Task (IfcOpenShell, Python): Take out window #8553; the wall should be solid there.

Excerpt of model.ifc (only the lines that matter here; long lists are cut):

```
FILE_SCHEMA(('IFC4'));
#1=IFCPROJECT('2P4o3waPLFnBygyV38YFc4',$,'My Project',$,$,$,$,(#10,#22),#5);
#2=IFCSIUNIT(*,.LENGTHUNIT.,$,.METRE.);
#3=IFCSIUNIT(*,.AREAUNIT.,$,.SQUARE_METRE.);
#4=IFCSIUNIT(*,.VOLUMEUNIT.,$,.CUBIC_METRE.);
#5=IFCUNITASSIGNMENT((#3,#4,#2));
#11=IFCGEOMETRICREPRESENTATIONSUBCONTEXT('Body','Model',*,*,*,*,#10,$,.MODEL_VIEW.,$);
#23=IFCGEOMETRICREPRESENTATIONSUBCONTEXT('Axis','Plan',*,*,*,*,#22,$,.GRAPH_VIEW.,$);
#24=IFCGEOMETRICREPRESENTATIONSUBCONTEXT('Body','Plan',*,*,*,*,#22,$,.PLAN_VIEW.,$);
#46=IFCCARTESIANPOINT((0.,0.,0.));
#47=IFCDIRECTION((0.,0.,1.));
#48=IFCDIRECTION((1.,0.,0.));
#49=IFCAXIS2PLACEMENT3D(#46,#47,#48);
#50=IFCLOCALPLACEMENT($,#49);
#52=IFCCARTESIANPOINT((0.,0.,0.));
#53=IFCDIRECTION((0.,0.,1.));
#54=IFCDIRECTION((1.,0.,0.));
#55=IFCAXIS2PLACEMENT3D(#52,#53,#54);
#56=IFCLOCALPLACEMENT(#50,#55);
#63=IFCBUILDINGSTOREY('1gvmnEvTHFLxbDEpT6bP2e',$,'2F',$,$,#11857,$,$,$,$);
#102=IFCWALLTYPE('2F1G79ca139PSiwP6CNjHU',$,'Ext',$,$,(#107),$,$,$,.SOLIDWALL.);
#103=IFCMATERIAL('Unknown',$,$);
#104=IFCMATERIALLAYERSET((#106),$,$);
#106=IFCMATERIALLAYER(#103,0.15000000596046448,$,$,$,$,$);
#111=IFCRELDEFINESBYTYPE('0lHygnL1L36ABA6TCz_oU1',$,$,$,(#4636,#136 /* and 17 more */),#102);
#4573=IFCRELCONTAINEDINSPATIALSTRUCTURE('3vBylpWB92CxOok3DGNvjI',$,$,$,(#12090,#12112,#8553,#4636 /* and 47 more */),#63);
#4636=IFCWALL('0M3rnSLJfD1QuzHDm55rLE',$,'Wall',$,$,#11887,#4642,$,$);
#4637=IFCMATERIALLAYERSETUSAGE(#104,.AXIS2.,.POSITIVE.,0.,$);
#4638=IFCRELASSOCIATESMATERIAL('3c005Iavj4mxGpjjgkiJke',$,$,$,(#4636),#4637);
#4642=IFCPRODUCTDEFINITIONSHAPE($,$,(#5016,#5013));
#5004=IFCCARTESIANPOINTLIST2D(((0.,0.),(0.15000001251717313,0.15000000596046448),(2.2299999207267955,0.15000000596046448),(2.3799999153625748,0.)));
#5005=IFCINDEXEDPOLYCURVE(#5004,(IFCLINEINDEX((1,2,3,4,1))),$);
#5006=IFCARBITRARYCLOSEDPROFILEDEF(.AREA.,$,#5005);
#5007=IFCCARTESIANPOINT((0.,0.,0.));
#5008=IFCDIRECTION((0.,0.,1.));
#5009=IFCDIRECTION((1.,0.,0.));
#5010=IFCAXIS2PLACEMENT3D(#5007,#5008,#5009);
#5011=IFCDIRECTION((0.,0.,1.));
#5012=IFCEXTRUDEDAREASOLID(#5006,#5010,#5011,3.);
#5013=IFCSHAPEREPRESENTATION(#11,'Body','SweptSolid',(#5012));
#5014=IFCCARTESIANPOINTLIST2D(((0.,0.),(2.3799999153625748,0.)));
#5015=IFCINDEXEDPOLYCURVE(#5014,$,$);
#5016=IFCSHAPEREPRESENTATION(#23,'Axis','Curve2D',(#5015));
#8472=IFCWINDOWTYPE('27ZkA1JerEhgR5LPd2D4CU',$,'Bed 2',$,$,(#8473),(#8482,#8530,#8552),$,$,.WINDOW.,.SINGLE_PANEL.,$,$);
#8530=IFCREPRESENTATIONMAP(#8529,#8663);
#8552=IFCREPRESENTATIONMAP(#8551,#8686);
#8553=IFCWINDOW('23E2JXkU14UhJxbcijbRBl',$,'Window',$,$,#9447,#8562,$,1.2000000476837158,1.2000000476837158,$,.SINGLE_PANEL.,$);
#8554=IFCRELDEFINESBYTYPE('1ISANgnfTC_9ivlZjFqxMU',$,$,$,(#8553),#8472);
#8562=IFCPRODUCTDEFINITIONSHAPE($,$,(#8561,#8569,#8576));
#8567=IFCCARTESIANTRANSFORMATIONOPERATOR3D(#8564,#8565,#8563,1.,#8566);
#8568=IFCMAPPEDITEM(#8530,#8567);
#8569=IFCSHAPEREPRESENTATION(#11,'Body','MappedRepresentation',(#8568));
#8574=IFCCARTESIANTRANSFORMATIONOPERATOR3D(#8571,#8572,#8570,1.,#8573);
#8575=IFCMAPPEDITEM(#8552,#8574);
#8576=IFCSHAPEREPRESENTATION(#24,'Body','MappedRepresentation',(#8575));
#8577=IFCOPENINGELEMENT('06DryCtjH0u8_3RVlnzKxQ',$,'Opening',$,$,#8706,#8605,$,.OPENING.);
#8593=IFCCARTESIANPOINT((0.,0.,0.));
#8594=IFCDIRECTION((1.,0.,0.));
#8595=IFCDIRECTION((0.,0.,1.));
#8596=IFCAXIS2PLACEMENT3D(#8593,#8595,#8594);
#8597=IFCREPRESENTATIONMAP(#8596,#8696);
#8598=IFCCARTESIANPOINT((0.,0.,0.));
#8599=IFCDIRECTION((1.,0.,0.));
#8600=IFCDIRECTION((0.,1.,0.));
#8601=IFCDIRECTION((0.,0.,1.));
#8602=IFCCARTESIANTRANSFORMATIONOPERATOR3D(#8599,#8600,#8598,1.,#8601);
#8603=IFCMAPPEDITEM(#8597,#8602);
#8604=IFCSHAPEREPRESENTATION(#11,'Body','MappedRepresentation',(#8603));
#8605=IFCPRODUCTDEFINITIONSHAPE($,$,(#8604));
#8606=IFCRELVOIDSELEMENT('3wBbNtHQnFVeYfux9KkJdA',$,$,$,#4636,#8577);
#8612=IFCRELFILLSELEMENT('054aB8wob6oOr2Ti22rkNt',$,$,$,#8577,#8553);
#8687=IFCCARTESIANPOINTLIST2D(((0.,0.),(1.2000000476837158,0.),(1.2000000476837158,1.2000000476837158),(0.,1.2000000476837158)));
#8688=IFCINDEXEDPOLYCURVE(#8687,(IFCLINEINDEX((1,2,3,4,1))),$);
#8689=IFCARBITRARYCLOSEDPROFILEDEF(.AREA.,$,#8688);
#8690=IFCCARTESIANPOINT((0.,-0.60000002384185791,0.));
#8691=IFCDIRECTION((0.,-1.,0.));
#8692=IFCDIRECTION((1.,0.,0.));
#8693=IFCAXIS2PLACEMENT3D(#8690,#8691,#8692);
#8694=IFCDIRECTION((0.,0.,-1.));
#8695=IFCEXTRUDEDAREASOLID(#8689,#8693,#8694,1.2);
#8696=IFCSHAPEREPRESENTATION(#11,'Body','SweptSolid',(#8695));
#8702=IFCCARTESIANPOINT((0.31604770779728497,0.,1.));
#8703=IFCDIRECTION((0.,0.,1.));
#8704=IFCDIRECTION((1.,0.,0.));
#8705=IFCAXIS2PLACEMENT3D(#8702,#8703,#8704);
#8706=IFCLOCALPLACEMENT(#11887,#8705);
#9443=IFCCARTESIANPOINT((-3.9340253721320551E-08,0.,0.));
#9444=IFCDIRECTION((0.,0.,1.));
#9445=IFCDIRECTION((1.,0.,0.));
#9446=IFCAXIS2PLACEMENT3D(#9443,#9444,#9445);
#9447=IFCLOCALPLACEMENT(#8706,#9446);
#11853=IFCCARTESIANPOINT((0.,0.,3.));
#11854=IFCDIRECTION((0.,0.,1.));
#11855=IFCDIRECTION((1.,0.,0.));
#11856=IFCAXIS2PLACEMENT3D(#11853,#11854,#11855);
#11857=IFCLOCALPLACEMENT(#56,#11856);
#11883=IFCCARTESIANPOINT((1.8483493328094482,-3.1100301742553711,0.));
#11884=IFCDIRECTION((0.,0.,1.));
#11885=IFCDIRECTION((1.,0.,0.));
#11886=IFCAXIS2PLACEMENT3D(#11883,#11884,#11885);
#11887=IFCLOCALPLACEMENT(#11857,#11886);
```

```python
import ifcopenshell
import ifcopenshell.api.feature
import ifcopenshell.api.root
import ifcopenshell.geom
import ifcopenshell.util.shape

model = ifcopenshell.open("model.ifc")
settings = ifcopenshell.geom.settings()


def volume(element):
    """Net volume in cubic metres, openings subtracted."""
    shape = ifcopenshell.geom.create_shape(settings, element)
    return ifcopenshell.util.shape.get_volume(shape.geometry)


window = model.by_guid("23E2JXkU14UhJxbcijbRBl")
opening = window.FillsVoids[0].RelatingOpeningElement
wall = opening.VoidsElements[0].RelatingBuildingElement
before = volume(wall)

ifcopenshell.api.root.remove_product(model, product=window)
ifcopenshell.api.feature.remove_feature(model, feature=opening)

after = volume(wall)

print(f"wall volume {before:.3f} -> {after:.3f} m3")

model.write("model_v2.ifc")
```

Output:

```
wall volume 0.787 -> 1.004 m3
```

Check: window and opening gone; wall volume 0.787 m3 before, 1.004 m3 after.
